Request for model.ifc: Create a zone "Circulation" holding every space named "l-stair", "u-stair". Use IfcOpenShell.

First a look at what the model holds.

```python
import ifcopenshell

model = ifcopenshell.open("model.ifc")
print(model.schema)
seen = {}
for space in model.by_type("IfcSpace"):
    seen[space.LongName] = seen.get(space.LongName, 0) + 1
for name, count in sorted(seen.items(), key=str):
    print(count, "x", name)
print("zones:", [z.Name for z in model.by_type("IfcZone")][:20])
```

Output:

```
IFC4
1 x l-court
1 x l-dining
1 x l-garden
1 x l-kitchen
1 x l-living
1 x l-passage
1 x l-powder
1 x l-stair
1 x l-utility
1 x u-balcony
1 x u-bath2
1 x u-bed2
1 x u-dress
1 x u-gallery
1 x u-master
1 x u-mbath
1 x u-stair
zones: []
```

```python
import ifcopenshell
import ifcopenshell.api.group
import ifcopenshell.api.root

model = ifcopenshell.open("model.ifc")

names = {"l-stair", "u-stair"}
spaces = [s for s in model.by_type("IfcSpace") if s.LongName in names]

zone = ifcopenshell.api.root.create_entity(model, ifc_class="IfcZone", name="Circulation")
ifcopenshell.api.group.assign_group(model, products=spaces, group=zone)
print(len(spaces), "spaces in", zone.Name)

model.write("model-out.ifc")
```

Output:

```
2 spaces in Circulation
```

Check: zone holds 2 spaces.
